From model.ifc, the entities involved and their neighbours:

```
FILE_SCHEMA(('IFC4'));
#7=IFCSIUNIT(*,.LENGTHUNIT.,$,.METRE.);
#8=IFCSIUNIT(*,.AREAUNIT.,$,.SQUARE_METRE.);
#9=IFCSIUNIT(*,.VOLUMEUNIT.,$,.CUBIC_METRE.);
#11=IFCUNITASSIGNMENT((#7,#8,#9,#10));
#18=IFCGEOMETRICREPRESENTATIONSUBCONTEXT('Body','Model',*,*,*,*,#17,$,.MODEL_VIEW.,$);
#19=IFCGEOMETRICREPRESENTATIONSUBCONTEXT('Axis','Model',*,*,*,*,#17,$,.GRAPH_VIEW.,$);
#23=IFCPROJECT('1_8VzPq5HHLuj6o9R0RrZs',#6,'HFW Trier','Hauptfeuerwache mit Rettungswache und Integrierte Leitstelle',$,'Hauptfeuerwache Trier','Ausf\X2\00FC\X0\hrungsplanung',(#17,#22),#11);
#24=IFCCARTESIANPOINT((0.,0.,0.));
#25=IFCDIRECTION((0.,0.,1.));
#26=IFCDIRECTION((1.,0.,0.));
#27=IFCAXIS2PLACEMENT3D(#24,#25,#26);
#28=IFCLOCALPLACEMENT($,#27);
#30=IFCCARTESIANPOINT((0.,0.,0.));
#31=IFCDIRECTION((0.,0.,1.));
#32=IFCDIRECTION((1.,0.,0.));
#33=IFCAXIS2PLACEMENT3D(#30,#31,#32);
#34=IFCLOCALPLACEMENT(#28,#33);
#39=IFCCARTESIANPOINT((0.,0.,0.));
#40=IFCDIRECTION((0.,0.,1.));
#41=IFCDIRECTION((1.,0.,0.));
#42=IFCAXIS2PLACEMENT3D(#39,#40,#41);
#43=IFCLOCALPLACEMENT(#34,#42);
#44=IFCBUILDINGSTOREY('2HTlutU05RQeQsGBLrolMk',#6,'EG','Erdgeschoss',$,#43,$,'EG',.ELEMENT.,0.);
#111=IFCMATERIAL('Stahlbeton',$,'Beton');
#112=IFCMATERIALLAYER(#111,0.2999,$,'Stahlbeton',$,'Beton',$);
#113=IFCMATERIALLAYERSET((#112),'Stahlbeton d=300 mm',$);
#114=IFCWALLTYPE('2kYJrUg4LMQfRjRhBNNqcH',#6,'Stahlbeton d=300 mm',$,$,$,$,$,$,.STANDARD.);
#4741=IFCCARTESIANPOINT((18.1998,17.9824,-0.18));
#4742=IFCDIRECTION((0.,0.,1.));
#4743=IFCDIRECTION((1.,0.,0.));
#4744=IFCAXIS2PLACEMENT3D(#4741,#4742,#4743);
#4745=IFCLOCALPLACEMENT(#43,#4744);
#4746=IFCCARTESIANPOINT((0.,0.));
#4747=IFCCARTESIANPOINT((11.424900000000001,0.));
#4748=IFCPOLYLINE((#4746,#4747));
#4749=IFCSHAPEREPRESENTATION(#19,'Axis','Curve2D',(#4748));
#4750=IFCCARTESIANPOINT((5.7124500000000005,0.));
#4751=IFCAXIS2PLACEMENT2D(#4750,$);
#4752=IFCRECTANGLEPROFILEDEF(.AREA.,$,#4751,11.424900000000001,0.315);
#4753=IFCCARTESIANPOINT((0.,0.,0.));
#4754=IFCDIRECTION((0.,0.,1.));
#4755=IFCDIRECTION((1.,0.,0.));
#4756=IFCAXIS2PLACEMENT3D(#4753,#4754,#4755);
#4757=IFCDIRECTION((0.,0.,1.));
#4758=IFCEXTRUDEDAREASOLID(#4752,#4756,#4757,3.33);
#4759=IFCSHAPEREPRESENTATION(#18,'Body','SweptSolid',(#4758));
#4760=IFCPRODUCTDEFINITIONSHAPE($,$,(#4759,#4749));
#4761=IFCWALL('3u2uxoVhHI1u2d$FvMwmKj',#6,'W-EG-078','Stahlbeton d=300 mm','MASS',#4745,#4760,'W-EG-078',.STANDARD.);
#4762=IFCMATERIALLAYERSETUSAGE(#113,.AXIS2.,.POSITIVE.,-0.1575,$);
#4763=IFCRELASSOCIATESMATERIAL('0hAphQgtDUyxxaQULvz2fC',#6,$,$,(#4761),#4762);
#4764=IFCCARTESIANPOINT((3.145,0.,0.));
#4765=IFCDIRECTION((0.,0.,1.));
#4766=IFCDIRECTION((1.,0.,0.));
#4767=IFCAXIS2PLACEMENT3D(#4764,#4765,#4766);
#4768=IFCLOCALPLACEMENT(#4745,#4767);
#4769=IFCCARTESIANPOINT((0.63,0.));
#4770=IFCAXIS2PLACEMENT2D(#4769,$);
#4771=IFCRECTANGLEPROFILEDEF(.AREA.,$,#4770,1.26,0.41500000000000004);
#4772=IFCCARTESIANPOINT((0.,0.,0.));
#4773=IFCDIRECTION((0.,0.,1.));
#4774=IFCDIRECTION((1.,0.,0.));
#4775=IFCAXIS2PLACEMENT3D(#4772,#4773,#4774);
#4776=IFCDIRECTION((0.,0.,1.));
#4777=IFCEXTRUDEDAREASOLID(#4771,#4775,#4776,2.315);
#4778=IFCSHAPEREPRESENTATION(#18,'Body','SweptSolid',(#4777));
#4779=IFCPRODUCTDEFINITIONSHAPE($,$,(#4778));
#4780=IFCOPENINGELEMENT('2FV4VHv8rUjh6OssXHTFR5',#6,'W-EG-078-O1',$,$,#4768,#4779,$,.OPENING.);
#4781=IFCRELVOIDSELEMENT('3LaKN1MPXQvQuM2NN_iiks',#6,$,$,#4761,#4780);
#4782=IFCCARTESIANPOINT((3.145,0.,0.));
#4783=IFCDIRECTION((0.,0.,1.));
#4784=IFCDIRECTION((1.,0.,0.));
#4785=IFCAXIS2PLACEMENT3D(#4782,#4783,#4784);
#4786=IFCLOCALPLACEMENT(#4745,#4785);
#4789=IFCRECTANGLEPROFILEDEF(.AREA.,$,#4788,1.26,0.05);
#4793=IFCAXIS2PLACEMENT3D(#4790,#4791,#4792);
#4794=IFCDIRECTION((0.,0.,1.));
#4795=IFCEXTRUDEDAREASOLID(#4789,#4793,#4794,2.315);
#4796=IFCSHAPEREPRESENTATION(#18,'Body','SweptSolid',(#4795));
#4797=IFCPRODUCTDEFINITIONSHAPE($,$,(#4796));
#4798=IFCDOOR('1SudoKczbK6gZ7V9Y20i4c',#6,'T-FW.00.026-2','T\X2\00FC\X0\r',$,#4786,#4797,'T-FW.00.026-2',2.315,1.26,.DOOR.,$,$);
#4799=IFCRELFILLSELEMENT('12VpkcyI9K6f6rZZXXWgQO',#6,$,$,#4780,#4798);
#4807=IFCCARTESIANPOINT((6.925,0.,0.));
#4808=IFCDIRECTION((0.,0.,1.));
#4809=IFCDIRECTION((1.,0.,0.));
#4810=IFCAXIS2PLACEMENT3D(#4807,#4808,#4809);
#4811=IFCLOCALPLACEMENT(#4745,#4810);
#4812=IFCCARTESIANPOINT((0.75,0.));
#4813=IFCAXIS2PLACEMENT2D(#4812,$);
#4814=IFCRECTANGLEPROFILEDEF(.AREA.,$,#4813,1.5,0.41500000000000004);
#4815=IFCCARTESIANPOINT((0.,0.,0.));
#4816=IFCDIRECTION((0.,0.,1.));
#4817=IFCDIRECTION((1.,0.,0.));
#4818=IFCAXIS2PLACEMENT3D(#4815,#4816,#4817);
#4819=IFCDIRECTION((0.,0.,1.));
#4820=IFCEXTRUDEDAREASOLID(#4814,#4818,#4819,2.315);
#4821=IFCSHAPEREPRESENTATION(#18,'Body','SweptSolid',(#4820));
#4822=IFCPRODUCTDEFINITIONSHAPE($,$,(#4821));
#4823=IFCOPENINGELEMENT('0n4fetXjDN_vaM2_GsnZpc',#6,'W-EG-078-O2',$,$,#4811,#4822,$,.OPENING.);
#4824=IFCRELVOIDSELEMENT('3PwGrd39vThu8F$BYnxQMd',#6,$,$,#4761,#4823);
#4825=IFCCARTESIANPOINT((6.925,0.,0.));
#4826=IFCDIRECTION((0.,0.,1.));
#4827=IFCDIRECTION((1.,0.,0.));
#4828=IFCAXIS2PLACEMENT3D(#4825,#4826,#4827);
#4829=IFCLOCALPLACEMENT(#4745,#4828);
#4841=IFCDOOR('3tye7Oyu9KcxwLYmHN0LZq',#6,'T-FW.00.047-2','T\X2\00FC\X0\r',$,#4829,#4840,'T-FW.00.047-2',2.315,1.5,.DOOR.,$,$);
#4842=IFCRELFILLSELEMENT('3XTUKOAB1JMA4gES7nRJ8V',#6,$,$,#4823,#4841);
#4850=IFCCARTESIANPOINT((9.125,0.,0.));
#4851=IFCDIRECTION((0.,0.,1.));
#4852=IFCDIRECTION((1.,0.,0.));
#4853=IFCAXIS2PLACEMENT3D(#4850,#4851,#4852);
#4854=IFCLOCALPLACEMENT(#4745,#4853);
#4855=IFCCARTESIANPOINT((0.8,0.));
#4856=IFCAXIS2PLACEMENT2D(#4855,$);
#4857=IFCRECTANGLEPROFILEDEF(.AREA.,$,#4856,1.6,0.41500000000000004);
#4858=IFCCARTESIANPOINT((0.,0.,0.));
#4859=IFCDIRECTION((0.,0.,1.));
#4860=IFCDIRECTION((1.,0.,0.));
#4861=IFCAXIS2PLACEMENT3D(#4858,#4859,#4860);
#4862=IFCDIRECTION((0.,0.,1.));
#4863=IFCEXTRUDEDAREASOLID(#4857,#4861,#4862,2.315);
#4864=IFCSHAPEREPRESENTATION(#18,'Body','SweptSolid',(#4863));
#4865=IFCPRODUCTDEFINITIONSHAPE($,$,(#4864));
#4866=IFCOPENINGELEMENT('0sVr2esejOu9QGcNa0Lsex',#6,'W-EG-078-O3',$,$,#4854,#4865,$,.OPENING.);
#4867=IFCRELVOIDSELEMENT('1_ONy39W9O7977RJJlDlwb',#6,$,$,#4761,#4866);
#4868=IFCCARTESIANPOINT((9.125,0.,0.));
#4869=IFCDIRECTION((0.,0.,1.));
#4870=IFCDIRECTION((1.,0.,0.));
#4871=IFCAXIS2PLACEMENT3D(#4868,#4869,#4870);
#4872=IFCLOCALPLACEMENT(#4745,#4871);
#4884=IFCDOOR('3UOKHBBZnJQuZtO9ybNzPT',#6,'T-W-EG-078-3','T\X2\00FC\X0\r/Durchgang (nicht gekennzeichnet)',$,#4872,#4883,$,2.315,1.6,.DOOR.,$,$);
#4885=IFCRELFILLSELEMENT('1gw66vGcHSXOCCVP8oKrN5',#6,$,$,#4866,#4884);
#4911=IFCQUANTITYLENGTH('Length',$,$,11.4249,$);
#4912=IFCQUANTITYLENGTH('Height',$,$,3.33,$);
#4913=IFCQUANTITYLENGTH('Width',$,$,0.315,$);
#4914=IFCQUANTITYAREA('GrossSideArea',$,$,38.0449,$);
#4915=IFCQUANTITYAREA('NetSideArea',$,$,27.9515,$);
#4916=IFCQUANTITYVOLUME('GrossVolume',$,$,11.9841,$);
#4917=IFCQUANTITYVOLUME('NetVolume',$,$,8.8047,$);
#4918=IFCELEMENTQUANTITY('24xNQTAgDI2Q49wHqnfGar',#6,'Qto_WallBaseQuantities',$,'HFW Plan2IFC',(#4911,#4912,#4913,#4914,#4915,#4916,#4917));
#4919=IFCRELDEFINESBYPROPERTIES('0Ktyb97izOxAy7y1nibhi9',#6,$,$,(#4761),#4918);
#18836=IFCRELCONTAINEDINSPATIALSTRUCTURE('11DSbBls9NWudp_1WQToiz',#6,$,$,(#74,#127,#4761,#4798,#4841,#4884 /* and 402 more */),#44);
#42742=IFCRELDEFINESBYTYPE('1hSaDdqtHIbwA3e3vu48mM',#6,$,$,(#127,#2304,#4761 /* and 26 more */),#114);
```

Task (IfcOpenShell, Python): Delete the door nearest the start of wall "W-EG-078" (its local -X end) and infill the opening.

```python
import ifcopenshell
import ifcopenshell.api.feature
import ifcopenshell.api.pset
import ifcopenshell.api.root
import ifcopenshell.geom
import ifcopenshell.util.element
import ifcopenshell.util.shape
import ifcopenshell.util.unit

model = ifcopenshell.open("model.ifc")
area_scale = ifcopenshell.util.unit.calculate_unit_scale(model, "AREAUNIT")
volume_scale = ifcopenshell.util.unit.calculate_unit_scale(model, "VOLUMEUNIT")
settings = ifcopenshell.geom.settings()


def volume(element):
    """Net volume in cubic metres, openings subtracted."""
    shape = ifcopenshell.geom.create_shape(settings, element)
    return ifcopenshell.util.shape.get_volume(shape.geometry)


door = model.by_guid("1SudoKczbK6gZ7V9Y20i4c")
opening = door.FillsVoids[0].RelatingOpeningElement
wall = opening.VoidsElements[0].RelatingBuildingElement
before = volume(wall)

ifcopenshell.api.root.remove_product(model, product=door)
ifcopenshell.api.feature.remove_feature(model, feature=opening)

after = volume(wall)
thickness = 0.315  # wall thickness in metres

# Update the wall's stored quantities.
qto = model.by_id(ifcopenshell.util.element.get_pset(wall, "Qto_WallBaseQuantities", should_inherit=False)["id"])
ifcopenshell.api.pset.edit_qto(model, qto=qto, properties={
    "NetSideArea": after / thickness / area_scale,
    "NetVolume": after / volume_scale,
})

print(f"wall volume {before:.3f} -> {after:.3f} m3")

model.write("model_rev.ifc")
```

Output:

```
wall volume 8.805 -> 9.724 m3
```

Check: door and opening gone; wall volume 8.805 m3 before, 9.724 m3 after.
